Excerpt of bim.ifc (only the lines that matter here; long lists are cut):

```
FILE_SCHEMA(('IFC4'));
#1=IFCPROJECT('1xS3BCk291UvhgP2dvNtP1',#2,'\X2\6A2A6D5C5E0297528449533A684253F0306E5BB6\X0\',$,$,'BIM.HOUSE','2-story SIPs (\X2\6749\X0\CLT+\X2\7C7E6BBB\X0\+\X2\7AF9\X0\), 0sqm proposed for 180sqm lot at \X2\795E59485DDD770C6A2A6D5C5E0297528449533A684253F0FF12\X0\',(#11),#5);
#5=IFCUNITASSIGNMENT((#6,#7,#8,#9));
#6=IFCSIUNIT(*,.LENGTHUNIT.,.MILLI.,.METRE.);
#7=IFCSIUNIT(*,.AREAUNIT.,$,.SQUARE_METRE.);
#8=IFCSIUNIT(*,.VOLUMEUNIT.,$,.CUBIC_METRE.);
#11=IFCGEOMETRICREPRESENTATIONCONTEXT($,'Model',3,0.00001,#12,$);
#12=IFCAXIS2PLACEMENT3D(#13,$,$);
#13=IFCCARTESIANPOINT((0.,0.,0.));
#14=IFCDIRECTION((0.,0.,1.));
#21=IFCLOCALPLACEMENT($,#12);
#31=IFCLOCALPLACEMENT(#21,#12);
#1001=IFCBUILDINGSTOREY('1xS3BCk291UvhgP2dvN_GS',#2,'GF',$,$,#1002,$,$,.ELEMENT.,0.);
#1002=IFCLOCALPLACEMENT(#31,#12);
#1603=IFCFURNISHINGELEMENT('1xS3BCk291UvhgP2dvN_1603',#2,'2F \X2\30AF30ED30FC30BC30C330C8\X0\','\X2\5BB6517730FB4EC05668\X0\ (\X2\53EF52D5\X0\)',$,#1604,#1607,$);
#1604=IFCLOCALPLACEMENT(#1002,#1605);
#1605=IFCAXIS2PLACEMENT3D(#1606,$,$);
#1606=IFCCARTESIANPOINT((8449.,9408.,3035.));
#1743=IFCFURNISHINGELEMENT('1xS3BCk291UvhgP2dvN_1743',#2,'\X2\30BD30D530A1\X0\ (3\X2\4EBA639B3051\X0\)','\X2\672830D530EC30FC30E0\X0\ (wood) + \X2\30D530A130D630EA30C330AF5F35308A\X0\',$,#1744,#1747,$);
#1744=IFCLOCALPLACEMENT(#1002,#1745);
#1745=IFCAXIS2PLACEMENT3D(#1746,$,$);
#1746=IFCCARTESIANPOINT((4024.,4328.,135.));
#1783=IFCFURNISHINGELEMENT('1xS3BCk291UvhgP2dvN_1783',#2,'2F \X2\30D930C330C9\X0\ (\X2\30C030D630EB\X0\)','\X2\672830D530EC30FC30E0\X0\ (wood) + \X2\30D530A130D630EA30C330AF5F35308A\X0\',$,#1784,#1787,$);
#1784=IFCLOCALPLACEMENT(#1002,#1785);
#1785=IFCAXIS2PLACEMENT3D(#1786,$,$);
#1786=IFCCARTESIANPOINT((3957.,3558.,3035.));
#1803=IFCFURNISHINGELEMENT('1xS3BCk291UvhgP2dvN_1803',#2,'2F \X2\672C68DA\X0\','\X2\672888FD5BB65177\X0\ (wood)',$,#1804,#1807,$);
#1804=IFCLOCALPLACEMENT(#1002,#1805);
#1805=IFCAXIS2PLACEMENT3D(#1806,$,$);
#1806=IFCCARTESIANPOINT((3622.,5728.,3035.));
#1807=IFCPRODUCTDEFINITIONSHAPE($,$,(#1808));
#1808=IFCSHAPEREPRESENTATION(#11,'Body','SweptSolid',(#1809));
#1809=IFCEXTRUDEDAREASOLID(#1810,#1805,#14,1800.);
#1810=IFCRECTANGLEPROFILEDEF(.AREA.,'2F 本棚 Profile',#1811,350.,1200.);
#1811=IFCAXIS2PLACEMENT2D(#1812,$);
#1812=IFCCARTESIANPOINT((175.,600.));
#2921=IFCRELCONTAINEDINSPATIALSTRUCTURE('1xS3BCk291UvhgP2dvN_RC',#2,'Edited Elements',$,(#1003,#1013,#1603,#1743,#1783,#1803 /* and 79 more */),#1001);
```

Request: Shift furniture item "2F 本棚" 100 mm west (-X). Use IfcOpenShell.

```python
import ifcopenshell
import ifcopenshell.api.geometry
import ifcopenshell.util.placement
import ifcopenshell.util.unit

model = ifcopenshell.open("bim.ifc")
unit_scale = ifcopenshell.util.unit.calculate_unit_scale(model)

item = model.by_id(1803)
matrix = ifcopenshell.util.placement.get_local_placement(item.ObjectPlacement)
matrix[0, 3] -= 0.1 / unit_scale
ifcopenshell.api.geometry.edit_object_placement(model, product=item, matrix=matrix, is_si=False)

print(ifcopenshell.util.placement.get_local_placement(item.ObjectPlacement).round(3) + 0.0)

model.write("bim_v2.ifc")
```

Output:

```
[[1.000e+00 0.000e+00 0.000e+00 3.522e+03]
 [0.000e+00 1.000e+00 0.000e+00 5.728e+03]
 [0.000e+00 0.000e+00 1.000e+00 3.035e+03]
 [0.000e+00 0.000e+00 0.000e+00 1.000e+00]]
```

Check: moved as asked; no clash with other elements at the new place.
